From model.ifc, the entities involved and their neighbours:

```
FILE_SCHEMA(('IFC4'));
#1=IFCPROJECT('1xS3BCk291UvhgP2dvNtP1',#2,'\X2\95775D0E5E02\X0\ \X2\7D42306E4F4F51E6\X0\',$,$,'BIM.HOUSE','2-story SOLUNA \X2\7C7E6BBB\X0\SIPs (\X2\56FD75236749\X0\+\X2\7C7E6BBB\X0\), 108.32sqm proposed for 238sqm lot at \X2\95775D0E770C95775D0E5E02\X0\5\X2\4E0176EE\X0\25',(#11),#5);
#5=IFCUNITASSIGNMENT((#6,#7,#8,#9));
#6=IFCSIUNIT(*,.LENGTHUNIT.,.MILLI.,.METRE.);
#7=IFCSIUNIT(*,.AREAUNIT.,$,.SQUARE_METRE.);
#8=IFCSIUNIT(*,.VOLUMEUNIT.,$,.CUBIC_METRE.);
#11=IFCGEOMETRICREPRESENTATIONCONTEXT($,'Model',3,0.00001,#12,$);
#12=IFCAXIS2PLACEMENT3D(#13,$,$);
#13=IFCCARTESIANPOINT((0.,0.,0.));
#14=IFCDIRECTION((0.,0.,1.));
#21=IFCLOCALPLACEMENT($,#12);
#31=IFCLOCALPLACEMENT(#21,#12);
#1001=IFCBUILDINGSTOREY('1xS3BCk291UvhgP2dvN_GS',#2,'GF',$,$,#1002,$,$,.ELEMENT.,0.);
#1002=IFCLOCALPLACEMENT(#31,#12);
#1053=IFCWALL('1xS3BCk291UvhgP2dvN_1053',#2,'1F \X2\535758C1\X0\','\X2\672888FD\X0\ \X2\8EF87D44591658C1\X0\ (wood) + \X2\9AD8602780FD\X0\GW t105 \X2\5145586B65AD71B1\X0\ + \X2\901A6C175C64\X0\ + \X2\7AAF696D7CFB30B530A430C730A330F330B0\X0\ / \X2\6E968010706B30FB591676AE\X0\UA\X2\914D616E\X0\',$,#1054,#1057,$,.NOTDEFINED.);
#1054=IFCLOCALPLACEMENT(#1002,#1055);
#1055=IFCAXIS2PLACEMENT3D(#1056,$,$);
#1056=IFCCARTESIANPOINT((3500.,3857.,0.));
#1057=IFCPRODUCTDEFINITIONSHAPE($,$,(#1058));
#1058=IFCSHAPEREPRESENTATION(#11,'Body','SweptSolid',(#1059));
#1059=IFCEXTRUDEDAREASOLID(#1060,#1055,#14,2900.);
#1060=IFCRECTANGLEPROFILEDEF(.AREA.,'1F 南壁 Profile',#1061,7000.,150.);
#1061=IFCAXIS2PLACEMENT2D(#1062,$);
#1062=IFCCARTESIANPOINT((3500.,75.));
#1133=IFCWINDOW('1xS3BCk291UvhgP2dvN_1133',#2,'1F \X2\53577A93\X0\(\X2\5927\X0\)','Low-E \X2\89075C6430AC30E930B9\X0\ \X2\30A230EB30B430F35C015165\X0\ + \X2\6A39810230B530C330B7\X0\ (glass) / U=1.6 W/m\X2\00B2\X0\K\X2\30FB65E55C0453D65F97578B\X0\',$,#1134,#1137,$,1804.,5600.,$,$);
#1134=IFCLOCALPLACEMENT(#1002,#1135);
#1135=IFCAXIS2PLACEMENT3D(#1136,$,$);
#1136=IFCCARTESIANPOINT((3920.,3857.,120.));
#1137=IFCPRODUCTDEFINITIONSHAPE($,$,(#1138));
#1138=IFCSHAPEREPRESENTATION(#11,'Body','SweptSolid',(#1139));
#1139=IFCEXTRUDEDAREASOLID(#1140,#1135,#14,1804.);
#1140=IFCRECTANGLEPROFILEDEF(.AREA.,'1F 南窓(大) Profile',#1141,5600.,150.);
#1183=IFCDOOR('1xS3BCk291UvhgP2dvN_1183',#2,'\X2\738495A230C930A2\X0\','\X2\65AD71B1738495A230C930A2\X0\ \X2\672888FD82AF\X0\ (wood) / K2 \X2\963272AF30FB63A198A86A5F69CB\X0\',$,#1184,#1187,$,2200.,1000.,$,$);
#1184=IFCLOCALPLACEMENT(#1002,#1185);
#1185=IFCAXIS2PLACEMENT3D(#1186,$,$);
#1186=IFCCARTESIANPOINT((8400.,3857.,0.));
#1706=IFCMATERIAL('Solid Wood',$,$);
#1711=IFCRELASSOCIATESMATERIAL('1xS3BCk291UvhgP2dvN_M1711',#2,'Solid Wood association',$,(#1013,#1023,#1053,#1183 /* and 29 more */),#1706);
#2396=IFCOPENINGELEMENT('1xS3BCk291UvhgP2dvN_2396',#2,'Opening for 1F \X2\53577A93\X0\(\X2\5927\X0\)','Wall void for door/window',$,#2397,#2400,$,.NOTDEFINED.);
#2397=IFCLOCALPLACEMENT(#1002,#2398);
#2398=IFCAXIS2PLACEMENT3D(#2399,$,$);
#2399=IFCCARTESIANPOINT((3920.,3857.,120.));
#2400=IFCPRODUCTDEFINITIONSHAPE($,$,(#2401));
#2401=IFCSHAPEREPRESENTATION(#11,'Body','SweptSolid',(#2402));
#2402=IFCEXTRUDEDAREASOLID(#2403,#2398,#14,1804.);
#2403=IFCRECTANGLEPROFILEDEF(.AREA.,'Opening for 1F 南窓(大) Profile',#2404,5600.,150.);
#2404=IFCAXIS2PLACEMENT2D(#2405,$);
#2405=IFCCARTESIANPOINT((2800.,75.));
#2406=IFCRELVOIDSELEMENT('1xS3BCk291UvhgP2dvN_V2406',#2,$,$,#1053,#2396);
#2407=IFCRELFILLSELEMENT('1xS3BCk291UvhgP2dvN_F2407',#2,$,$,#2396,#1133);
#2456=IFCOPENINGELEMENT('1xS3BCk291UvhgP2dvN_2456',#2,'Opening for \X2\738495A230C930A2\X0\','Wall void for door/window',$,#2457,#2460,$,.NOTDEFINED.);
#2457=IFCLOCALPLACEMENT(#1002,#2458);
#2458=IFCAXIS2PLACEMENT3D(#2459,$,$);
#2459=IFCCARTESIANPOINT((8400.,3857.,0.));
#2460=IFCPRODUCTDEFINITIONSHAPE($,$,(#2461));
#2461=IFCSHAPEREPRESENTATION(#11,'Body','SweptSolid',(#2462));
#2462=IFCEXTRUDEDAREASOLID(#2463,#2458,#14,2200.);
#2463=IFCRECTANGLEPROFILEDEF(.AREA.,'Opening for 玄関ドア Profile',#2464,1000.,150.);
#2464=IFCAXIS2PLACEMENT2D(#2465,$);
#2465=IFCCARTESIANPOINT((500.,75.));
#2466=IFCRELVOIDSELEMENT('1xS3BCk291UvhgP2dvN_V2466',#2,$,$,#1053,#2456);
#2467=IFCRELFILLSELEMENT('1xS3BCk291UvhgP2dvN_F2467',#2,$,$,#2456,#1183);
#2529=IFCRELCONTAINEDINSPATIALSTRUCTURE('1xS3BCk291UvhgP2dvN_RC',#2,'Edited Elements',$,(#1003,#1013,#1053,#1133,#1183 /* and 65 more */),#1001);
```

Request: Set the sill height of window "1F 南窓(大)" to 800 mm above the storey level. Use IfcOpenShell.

```python
import numpy as np
import ifcopenshell
import ifcopenshell.api.geometry
import ifcopenshell.geom
import ifcopenshell.util.element
import ifcopenshell.util.placement
import ifcopenshell.util.shape
import ifcopenshell.util.unit

model = ifcopenshell.open("model.ifc")
unit_scale = ifcopenshell.util.unit.calculate_unit_scale(model)

window = model.by_id(1133)
opening = window.FillsVoids[0].RelatingOpeningElement
storey = ifcopenshell.util.element.get_container(window, ifc_class="IfcBuildingStorey")
level = ifcopenshell.util.placement.get_local_placement(storey.ObjectPlacement)[2, 3]

# The opening's origin need not be at the sill, so measure its lowest point.
shape = ifcopenshell.geom.create_shape(ifcopenshell.geom.settings(), opening)
bottom = ifcopenshell.util.shape.get_shape_bottom_elevation(shape, shape.geometry) / unit_scale
dz = level + 0.8 / unit_scale - bottom

shift = np.array([0.0, 0.0, dz])
# The window is not placed relative to its opening, so move both.
for product in (opening, window):
    matrix = ifcopenshell.util.placement.get_local_placement(product.ObjectPlacement)
    matrix[:3, 3] += shift
    ifcopenshell.api.geometry.edit_object_placement(model, product=product, matrix=matrix, is_si=False)

print(f"moved by {dz * unit_scale:+.3f} m")

model.write("model_edited.ifc")
```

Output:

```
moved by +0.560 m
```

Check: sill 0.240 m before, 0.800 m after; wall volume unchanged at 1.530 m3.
